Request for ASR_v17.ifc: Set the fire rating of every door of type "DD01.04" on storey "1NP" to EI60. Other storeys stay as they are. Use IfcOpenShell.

First a look at what the model holds.

```python
import ifcopenshell
import ifcopenshell.util.element

model = ifcopenshell.open("ASR_v17.ifc")
print(model.schema)
storey = next(s for s in model.by_type("IfcBuildingStorey") if s.Name == "1NP")
doors = [e for e in ifcopenshell.util.element.get_decomposition(storey) if e.is_a("IfcDoor")]
seen = {}
for e in doors:
    element_type = ifcopenshell.util.element.get_type(e)
    key = (element_type.Name if element_type != e and element_type else None, ifcopenshell.util.element.get_pset(e, "Pset_DoorCommon", "FireRating"))
    seen[key] = seen.get(key, 0) + 1
for (name, value), count in sorted(seen.items(), key=str):
    print(count, "x", name, "|", value)
```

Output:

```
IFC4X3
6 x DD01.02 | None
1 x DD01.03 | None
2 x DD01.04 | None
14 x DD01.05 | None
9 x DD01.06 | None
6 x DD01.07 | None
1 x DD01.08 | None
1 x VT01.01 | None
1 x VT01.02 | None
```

```python
import ifcopenshell
import ifcopenshell.api.pset
import ifcopenshell.util.element

model = ifcopenshell.open("ASR_v17.ifc")

storey = next(s for s in model.by_type("IfcBuildingStorey") if s.Name == "1NP")
doors = [e for e in ifcopenshell.util.element.get_decomposition(storey) if e.is_a("IfcDoor")]

count = 0
for e in doors:
    element_type = ifcopenshell.util.element.get_type(e)
    if element_type in (None, e) or element_type.Name != "DD01.04":
        continue
    # add_pset returns the element's existing set when there is one.
    pset = ifcopenshell.api.pset.add_pset(model, product=e, name="Pset_DoorCommon")
    ifcopenshell.api.pset.edit_pset(model, pset=pset, properties={"FireRating": "EI60"})
    count += 1

print(count, "doors updated")

model.write("ASR_v17-out.ifc")
```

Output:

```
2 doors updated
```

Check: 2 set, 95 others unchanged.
